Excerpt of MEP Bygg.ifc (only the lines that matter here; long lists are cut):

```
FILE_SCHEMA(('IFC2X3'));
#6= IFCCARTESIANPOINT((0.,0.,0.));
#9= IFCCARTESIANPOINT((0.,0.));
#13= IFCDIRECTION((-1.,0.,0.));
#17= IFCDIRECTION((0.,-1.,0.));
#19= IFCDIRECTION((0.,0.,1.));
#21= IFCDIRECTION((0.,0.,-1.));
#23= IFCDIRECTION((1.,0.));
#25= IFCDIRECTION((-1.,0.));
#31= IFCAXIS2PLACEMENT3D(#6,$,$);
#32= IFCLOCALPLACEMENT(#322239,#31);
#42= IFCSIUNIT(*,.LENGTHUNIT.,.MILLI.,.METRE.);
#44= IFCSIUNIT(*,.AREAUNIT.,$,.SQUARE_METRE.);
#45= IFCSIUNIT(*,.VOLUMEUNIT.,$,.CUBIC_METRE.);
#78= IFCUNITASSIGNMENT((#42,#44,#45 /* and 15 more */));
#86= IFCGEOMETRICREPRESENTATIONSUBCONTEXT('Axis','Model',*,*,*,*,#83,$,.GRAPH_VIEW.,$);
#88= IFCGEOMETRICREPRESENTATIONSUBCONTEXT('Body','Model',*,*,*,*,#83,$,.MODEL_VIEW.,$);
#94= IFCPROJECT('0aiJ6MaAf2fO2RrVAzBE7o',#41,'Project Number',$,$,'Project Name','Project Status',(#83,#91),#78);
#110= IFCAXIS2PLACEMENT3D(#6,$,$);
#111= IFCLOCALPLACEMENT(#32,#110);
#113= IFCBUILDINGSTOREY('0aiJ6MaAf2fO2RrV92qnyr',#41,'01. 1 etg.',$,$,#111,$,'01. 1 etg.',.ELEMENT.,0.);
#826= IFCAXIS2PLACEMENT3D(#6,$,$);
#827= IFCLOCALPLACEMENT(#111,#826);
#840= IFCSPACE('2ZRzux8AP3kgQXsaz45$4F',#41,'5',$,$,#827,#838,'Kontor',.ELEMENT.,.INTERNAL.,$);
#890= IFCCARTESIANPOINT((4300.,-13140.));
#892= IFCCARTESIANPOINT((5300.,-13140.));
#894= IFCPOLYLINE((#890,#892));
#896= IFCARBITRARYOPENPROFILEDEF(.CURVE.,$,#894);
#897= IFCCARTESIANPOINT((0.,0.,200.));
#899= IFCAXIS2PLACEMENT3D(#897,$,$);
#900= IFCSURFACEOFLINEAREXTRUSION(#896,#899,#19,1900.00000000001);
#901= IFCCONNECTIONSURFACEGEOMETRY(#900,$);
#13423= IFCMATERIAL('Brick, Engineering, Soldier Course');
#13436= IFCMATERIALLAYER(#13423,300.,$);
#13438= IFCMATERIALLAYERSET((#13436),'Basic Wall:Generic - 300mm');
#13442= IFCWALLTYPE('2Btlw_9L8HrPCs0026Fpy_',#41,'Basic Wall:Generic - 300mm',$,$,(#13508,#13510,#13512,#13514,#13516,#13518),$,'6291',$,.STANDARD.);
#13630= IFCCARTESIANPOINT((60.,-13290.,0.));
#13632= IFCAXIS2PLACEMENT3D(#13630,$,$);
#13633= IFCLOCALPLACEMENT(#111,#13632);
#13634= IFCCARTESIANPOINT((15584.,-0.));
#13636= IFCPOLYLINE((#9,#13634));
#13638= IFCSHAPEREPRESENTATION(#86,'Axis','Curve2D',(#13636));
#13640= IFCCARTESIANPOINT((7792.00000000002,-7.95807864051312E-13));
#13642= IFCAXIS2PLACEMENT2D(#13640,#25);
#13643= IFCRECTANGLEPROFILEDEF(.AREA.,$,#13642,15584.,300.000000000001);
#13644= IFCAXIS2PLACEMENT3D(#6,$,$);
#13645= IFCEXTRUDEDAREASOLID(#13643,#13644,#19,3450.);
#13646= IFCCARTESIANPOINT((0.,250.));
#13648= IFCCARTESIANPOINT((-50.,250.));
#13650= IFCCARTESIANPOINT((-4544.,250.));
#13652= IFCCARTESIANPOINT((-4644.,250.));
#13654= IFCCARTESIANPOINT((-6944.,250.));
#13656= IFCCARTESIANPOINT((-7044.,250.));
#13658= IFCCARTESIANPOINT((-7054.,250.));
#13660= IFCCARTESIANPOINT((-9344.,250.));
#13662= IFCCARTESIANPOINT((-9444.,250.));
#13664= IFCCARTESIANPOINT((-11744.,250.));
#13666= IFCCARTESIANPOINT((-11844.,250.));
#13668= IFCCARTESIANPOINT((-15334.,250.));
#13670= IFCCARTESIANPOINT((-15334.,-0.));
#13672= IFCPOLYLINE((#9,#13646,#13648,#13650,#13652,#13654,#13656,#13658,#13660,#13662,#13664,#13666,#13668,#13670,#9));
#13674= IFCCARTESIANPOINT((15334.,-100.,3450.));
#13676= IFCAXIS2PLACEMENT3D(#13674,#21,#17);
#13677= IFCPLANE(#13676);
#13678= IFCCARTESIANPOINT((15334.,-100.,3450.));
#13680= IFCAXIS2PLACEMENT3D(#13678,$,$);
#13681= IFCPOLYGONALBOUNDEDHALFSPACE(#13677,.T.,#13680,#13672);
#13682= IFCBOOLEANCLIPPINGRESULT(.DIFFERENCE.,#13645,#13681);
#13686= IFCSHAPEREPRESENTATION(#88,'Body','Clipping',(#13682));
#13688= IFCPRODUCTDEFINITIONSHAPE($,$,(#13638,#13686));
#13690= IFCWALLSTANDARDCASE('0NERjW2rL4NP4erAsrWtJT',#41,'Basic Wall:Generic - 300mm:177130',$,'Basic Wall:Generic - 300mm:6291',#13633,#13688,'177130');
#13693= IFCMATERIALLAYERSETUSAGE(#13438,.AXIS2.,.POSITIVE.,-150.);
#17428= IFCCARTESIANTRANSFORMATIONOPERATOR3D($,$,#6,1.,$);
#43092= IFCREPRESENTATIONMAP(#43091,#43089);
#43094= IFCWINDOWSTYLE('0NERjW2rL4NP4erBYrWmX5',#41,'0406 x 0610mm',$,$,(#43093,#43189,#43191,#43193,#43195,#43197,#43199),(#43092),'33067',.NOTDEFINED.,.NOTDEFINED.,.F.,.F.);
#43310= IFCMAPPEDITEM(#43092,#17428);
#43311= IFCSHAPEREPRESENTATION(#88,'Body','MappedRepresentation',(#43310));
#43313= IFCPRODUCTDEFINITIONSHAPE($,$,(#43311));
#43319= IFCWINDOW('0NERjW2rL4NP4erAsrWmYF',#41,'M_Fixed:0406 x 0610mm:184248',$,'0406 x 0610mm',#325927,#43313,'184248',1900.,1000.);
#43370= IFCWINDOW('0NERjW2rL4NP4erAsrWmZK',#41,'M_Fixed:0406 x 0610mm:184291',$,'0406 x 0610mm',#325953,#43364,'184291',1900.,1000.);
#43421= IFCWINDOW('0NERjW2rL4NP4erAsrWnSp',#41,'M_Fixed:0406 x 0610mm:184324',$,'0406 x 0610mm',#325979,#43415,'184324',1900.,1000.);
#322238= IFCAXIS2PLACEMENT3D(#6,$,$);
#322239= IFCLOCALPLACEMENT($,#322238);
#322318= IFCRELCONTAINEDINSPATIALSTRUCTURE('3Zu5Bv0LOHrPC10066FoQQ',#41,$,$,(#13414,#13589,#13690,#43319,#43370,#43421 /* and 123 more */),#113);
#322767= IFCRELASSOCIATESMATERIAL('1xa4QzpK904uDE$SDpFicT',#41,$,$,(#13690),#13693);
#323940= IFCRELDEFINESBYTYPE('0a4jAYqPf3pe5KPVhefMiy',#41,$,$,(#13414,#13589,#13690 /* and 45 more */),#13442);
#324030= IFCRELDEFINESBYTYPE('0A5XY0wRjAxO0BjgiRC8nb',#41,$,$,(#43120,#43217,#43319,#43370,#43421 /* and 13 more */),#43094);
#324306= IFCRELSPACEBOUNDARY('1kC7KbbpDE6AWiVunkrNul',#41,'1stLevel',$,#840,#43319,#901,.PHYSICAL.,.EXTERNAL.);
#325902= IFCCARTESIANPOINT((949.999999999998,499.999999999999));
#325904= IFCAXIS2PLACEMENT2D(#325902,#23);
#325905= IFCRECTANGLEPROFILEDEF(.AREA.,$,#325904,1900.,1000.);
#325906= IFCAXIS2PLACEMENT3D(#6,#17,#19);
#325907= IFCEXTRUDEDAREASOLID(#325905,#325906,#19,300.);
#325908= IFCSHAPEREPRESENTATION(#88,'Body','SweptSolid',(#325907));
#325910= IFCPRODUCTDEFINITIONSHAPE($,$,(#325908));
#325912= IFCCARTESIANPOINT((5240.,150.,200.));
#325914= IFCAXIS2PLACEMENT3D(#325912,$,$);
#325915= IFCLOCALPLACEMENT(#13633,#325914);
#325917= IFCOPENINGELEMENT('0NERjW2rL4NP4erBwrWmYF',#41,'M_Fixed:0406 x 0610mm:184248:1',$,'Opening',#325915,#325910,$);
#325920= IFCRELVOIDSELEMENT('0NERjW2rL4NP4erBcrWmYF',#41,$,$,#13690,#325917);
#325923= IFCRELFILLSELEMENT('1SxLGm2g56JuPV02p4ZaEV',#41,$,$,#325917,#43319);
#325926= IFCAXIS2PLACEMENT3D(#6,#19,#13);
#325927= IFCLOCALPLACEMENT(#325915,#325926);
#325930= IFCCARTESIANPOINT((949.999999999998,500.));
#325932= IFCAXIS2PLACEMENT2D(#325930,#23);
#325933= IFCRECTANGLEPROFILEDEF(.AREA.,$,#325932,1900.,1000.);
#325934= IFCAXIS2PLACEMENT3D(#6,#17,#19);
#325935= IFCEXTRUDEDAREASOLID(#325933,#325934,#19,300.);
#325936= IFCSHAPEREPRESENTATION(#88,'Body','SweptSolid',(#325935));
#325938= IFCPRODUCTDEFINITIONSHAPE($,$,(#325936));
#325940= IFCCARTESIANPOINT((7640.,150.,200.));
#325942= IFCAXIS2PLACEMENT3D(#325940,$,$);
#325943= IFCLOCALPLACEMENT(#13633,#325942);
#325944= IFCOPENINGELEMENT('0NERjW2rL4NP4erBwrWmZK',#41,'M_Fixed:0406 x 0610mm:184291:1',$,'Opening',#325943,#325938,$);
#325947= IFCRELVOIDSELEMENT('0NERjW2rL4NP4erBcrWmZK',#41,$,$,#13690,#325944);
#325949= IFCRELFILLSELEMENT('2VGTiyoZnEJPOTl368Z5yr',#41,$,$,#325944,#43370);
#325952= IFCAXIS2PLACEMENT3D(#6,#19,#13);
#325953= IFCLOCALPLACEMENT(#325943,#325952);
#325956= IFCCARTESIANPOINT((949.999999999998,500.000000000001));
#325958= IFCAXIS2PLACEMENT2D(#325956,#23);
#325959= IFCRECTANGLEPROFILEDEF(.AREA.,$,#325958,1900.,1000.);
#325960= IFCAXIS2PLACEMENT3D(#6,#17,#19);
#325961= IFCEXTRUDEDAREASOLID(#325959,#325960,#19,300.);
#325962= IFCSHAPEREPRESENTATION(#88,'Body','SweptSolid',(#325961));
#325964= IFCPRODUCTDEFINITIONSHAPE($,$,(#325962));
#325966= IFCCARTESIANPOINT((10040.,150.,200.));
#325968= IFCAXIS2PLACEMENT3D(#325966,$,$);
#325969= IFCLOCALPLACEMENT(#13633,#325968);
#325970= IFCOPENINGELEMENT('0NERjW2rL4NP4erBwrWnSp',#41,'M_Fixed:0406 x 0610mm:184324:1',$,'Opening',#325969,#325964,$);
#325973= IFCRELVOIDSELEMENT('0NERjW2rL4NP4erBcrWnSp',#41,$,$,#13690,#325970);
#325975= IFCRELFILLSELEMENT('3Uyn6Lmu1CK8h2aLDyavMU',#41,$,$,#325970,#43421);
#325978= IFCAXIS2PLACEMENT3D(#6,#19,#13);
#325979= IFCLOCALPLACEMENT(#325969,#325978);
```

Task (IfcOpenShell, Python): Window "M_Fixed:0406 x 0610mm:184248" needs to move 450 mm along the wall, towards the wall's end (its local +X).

```python
import numpy as np
import ifcopenshell
import ifcopenshell.api.geometry
import ifcopenshell.util.placement
import ifcopenshell.util.unit

model = ifcopenshell.open("MEP Bygg.ifc")
unit_scale = ifcopenshell.util.unit.calculate_unit_scale(model)

window = model.by_guid("0NERjW2rL4NP4erAsrWmYF")
opening = window.FillsVoids[0].RelatingOpeningElement
wall = opening.VoidsElements[0].RelatingBuildingElement

wall_matrix = ifcopenshell.util.placement.get_local_placement(wall.ObjectPlacement)
shift = wall_matrix[:3, 0] * 0.45 / unit_scale
before = ifcopenshell.util.placement.get_local_placement(window.ObjectPlacement)[:3, 3].copy()

# The window is placed relative to its opening, so it follows when the opening moves.
matrix = ifcopenshell.util.placement.get_local_placement(opening.ObjectPlacement)
matrix[:3, 3] += shift
ifcopenshell.api.geometry.edit_object_placement(
    model, product=opening, matrix=matrix, is_si=False, should_transform_children=True
)

# Space boundary surfaces are stored in each space's coordinates; move them too.
for rel in window.ProvidesBoundaries:
    if not rel.ConnectionGeometry:
        continue
    surface = rel.ConnectionGeometry.SurfaceOnRelatingElement
    space_matrix = ifcopenshell.util.placement.get_local_placement(rel.RelatingSpace.ObjectPlacement)
    point = np.array(surface.Position.Location.Coordinates) + space_matrix[:3, :3].T @ shift
    surface.Position = model.createIfcAxis2Placement3D(
        model.createIfcCartesianPoint(point.tolist()), surface.Position.Axis, surface.Position.RefDirection
    )

after = ifcopenshell.util.placement.get_local_placement(window.ObjectPlacement)[:3, 3]
print("window moved by", (after - before).round(3) + 0.0)

model.write("MEP Bygg_v2.ifc")
```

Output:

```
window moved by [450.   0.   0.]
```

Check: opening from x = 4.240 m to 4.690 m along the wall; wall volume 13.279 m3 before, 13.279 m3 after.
